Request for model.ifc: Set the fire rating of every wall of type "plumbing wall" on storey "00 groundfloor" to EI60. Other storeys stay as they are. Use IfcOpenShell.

First a look at what the model holds.

```python
import ifcopenshell
import ifcopenshell.util.element

model = ifcopenshell.open("model.ifc")
print(model.schema)
storey = next(s for s in model.by_type("IfcBuildingStorey") if s.Name == "00 groundfloor")
walls = [e for e in ifcopenshell.util.element.get_decomposition(storey) if e.is_a("IfcWall")]
seen = {}
for e in walls:
    element_type = ifcopenshell.util.element.get_type(e)
    key = (element_type.Name if element_type != e and element_type else None, ifcopenshell.util.element.get_pset(e, "Pset_WallCommon", "FireRating"))
    seen[key] = seen.get(key, 0) + 1
for (name, value), count in sorted(seen.items(), key=str):
    print(count, "x", name, "|", value)
```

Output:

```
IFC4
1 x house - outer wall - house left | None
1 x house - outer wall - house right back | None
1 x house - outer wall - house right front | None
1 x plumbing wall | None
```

```python
import ifcopenshell
import ifcopenshell.api.pset
import ifcopenshell.util.element

model = ifcopenshell.open("model.ifc")

storey = next(s for s in model.by_type("IfcBuildingStorey") if s.Name == "00 groundfloor")
walls = [e for e in ifcopenshell.util.element.get_decomposition(storey) if e.is_a("IfcWall")]

count = 0
for e in walls:
    element_type = ifcopenshell.util.element.get_type(e)
    if element_type in (None, e) or element_type.Name != "plumbing wall":
        continue
    # add_pset returns the element's existing set when there is one.
    pset = ifcopenshell.api.pset.add_pset(model, product=e, name="Pset_WallCommon")
    ifcopenshell.api.pset.edit_pset(model, pset=pset, properties={"FireRating": "EI60"})
    count += 1

print(count, "walls updated")

model.write("model_edited.ifc")
```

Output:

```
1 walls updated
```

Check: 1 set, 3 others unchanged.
